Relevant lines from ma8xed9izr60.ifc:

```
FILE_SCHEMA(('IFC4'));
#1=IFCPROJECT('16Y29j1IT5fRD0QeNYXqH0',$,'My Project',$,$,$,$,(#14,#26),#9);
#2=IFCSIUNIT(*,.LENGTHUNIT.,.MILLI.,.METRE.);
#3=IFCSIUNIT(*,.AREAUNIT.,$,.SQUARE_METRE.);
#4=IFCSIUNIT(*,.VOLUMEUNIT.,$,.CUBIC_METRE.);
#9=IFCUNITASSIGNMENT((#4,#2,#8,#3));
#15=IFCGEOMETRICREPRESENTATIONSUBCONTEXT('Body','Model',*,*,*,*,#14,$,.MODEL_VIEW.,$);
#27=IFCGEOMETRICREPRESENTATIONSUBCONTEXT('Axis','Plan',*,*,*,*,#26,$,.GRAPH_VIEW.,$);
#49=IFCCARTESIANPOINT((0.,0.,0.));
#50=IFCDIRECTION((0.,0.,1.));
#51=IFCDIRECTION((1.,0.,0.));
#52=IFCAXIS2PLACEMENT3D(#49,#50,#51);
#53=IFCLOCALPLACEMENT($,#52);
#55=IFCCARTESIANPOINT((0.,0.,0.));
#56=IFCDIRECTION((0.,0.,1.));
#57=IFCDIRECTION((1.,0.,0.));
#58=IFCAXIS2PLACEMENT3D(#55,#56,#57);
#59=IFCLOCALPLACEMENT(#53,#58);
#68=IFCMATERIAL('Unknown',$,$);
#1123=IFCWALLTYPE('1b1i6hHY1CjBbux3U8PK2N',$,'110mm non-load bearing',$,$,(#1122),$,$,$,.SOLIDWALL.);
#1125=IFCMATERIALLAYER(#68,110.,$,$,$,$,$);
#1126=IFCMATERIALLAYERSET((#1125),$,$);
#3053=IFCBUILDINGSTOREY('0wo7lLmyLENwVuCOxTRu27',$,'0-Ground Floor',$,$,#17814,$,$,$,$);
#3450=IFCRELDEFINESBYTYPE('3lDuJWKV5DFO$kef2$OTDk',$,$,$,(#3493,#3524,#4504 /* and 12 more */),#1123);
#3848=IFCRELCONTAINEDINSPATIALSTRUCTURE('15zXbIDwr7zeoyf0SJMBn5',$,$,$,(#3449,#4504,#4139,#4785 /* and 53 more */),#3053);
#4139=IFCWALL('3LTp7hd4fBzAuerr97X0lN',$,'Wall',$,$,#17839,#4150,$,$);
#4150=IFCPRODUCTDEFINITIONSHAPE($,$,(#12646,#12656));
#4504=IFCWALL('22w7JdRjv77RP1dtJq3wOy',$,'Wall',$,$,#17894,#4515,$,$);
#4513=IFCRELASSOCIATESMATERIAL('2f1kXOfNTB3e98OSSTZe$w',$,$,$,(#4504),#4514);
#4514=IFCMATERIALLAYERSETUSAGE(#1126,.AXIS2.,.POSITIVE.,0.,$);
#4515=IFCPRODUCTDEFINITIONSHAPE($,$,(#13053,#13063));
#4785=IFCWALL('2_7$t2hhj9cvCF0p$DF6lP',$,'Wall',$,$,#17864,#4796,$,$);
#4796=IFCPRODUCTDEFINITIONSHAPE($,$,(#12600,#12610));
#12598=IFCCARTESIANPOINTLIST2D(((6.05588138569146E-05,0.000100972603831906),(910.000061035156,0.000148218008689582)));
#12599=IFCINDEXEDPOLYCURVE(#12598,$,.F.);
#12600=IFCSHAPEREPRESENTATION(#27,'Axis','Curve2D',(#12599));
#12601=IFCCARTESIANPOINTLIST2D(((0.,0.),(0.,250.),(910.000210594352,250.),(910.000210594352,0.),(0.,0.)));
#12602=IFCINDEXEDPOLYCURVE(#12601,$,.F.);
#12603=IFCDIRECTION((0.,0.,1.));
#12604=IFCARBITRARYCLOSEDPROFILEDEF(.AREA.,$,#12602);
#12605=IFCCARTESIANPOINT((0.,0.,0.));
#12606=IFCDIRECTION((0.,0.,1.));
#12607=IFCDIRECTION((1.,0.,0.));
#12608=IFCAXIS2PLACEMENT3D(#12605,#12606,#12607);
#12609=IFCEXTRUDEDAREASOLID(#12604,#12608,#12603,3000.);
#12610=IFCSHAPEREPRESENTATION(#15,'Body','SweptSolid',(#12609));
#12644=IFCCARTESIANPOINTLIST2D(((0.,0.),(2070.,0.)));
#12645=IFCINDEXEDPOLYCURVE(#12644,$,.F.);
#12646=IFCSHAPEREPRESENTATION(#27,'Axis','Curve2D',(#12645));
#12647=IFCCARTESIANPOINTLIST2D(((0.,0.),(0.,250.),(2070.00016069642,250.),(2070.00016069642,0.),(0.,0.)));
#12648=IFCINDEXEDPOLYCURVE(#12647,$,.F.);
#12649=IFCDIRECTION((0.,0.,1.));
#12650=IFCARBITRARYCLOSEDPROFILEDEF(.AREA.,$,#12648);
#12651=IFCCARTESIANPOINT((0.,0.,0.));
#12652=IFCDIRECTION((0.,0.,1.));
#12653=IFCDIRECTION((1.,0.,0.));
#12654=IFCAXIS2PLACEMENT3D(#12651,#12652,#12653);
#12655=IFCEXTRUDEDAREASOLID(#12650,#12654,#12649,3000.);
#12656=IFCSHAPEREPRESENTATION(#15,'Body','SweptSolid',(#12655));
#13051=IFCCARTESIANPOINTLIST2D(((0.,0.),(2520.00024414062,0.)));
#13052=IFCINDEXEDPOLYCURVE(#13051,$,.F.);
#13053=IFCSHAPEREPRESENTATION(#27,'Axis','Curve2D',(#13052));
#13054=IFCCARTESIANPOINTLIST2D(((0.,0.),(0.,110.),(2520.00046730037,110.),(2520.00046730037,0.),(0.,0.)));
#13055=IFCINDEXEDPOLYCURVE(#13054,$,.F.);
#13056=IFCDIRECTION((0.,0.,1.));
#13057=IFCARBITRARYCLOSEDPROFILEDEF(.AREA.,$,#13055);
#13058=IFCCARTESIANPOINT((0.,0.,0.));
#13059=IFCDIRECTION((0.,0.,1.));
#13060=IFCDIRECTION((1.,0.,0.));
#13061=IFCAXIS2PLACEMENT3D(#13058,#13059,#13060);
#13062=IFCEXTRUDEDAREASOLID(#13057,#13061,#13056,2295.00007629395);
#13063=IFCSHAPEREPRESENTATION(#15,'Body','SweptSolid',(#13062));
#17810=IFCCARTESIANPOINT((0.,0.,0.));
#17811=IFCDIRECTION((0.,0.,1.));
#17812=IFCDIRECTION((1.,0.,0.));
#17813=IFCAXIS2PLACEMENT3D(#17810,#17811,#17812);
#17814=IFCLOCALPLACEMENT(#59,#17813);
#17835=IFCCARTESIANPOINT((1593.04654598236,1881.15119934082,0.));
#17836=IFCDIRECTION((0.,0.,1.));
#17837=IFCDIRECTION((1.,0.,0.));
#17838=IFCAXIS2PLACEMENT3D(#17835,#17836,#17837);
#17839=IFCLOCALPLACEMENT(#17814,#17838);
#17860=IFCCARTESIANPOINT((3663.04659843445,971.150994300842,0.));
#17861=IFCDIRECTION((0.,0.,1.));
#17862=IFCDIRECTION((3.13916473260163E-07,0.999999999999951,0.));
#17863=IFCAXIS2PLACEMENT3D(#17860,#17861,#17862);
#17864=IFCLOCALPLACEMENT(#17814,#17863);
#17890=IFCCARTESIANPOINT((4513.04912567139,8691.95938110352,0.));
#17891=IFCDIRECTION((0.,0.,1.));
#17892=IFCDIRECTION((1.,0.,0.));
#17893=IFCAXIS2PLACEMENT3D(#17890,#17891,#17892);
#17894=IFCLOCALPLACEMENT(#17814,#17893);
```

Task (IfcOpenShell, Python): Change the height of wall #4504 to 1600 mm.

```python
import ifcopenshell
import ifcopenshell.geom
import ifcopenshell.util.representation
import ifcopenshell.util.shape
import ifcopenshell.util.unit

model = ifcopenshell.open("ma8xed9izr60.ifc")
unit_scale = ifcopenshell.util.unit.calculate_unit_scale(model)
settings = ifcopenshell.geom.settings()


def volume(element):
    """Net volume in cubic metres, openings subtracted."""
    shape = ifcopenshell.geom.create_shape(settings, element)
    return ifcopenshell.util.shape.get_volume(shape.geometry)


wall = model.by_guid("22w7JdRjv77RP1dtJq3wOy")
before = volume(wall)

body = ifcopenshell.util.representation.get_representation(wall, "Model", "Body")
solid = body.Items[0]
old_height = solid.Depth
solid.Depth = 1.6 / unit_scale
after = volume(wall)

print(f"height {old_height:g} -> {solid.Depth:g}, volume {before:.3f} -> {after:.3f} m3")

model.write("ma8xed9izr60_updated.ifc")
```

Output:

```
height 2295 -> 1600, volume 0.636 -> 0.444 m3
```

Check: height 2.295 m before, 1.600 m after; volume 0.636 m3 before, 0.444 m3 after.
